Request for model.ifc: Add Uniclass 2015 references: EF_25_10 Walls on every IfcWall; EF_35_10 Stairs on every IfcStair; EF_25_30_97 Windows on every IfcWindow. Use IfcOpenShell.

First a look at what the model holds.

```python
import ifcopenshell

model = ifcopenshell.open("model.ifc")
print(model.schema)
print("classifications:", [c.Name for c in model.by_type("IfcClassification")])
for ifc_class in ("IfcDoor", "IfcRoof", "IfcStair", "IfcWall", "IfcWindow"):
    print(ifc_class, len(model.by_type(ifc_class)))
```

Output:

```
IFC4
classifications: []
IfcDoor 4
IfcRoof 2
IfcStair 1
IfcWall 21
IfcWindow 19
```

```python
import ifcopenshell
import ifcopenshell.api.classification

model = ifcopenshell.open("model.ifc")

system = ifcopenshell.api.classification.add_classification(model, classification="Uniclass 2015")

codes = {
    "IfcWall": ("EF_25_10", "Walls"),
    "IfcStair": ("EF_35_10", "Stairs"),
    "IfcWindow": ("EF_25_30_97", "Windows"),
}
for ifc_class, (code, name) in codes.items():
    products = model.by_type(ifc_class)
    ifcopenshell.api.classification.add_reference(
        model, products=products, classification=system, identification=code, name=name
    )
    print(code, len(products))

model.write("model_v2.ifc")
```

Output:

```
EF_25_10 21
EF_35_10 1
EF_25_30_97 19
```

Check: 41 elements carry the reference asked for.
